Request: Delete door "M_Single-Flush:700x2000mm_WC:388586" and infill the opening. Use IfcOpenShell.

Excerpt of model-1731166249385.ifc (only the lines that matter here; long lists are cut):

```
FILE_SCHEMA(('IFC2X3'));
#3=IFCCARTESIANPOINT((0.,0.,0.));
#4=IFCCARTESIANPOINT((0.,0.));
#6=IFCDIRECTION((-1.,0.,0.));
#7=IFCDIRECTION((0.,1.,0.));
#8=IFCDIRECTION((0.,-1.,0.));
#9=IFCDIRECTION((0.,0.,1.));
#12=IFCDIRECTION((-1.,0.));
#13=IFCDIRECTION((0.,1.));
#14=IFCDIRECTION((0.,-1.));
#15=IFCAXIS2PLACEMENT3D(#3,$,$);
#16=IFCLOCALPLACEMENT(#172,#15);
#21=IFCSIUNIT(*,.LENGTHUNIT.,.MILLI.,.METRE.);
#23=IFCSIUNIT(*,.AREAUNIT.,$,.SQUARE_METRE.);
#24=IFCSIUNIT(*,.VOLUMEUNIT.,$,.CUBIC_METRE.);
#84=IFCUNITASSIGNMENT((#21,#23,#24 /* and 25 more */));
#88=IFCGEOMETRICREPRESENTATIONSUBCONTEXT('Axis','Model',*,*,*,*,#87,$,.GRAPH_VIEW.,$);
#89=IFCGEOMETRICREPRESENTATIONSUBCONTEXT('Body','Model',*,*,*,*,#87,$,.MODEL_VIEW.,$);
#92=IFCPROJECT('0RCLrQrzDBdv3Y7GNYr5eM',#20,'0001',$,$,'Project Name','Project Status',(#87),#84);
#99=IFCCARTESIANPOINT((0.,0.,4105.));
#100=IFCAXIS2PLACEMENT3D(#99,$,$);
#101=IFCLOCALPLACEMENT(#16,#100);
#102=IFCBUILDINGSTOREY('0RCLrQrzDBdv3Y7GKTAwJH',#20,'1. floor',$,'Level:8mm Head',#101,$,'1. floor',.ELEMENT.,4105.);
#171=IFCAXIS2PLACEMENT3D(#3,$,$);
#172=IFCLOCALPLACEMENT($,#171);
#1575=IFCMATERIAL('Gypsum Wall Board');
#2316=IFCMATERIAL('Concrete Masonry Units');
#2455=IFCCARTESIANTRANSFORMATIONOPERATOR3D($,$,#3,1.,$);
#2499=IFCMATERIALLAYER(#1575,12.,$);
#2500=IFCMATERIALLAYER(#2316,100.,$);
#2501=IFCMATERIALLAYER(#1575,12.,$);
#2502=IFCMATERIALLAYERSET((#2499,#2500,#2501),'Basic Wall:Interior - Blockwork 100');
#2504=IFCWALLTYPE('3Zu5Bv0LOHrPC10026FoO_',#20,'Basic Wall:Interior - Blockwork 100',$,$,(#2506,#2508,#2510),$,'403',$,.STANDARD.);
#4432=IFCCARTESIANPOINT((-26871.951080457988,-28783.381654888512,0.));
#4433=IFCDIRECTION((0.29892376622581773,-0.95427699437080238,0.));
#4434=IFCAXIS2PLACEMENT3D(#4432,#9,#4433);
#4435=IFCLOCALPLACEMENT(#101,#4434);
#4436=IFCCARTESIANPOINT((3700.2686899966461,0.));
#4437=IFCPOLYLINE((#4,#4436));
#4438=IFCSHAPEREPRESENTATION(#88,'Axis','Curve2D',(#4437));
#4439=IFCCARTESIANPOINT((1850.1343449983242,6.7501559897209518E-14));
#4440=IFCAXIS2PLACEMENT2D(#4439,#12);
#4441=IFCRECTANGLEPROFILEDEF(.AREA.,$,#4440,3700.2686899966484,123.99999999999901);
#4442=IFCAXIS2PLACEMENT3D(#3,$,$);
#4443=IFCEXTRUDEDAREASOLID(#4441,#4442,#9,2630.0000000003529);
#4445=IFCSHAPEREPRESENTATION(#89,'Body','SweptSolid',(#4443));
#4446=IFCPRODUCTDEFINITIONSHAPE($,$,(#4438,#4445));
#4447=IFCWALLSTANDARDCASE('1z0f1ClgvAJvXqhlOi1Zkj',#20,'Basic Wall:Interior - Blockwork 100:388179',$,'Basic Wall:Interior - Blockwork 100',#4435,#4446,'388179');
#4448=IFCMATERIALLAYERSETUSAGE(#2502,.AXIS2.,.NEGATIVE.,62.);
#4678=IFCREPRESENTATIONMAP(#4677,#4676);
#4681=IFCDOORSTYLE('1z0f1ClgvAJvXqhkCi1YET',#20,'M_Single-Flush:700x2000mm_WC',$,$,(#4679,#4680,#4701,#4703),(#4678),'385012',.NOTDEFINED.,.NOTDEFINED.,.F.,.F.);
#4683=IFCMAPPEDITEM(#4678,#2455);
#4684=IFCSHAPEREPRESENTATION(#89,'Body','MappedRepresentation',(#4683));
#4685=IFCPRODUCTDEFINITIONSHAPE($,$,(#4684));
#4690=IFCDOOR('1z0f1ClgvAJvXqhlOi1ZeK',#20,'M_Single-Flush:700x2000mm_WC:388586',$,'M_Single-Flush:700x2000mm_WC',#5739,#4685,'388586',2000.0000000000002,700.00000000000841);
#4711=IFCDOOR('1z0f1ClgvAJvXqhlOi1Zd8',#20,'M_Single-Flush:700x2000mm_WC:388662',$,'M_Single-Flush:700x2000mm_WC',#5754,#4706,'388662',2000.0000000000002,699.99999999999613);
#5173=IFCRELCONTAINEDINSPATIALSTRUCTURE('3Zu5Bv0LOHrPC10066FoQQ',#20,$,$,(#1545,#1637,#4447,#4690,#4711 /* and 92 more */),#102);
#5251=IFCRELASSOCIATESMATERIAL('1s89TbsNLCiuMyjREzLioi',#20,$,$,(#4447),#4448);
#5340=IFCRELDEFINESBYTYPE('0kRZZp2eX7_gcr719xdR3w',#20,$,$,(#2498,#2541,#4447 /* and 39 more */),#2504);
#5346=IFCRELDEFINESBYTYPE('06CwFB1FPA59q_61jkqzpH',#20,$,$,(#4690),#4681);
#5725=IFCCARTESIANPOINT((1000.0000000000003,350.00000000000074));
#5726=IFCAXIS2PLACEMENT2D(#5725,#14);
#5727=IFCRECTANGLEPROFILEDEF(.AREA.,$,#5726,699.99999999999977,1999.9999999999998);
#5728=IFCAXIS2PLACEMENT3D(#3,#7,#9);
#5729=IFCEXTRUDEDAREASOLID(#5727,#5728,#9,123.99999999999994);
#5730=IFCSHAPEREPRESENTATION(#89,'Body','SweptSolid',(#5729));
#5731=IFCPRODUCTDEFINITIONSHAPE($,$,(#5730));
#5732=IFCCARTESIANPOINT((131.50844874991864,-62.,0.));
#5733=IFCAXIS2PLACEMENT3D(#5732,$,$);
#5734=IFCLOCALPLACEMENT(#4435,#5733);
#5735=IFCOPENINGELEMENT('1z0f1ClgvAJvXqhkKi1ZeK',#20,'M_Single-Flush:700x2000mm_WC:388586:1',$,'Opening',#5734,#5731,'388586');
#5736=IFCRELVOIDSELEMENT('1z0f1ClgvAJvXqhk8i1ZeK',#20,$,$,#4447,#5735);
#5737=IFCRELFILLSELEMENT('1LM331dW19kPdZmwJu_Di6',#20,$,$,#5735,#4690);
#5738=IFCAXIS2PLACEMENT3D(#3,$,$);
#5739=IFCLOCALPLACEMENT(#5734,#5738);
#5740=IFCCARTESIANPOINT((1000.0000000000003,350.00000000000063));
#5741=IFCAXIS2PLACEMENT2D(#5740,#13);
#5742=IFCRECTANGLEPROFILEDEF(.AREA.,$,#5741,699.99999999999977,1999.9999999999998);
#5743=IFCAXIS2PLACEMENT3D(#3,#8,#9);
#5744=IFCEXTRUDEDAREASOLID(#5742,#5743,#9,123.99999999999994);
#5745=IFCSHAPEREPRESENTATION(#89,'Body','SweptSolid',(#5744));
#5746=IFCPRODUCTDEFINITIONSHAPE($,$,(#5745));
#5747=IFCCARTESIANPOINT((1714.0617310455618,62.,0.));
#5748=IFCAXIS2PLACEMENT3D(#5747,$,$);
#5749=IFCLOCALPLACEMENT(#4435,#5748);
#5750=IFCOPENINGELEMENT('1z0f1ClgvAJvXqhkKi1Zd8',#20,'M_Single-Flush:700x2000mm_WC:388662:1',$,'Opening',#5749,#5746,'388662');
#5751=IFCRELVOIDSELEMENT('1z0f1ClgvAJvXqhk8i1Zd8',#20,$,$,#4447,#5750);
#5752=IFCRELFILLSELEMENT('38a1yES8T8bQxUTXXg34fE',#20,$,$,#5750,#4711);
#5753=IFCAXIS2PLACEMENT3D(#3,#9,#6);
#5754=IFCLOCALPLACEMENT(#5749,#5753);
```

```python
import ifcopenshell
import ifcopenshell.api.feature
import ifcopenshell.api.root
import ifcopenshell.geom
import ifcopenshell.util.shape

model = ifcopenshell.open("model-1731166249385.ifc")
settings = ifcopenshell.geom.settings()


def volume(element):
    """Net volume in cubic metres, openings subtracted."""
    shape = ifcopenshell.geom.create_shape(settings, element)
    return ifcopenshell.util.shape.get_volume(shape.geometry)


door = model.by_guid("1z0f1ClgvAJvXqhlOi1ZeK")
opening = door.FillsVoids[0].RelatingOpeningElement
wall = opening.VoidsElements[0].RelatingBuildingElement
before = volume(wall)

ifcopenshell.api.root.remove_product(model, product=door)
ifcopenshell.api.feature.remove_feature(model, feature=opening)

after = volume(wall)

print(f"wall volume {before:.3f} -> {after:.3f} m3")

model.write("model-1731166249385_updated.ifc")
```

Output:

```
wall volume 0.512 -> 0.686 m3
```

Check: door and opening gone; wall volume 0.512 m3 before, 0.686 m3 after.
